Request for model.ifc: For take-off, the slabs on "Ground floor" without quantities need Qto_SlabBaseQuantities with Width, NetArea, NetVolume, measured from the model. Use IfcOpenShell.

First a look at what the model holds.

```python
import ifcopenshell
import ifcopenshell.util.element
import ifcopenshell.util.unit

model = ifcopenshell.open("model.ifc")
print(model.schema)
for unit_type in ("LENGTHUNIT", "AREAUNIT", "VOLUMEUNIT"):
    print(unit_type, ifcopenshell.util.unit.calculate_unit_scale(model, unit_type))
storey = next(s for s in model.by_type("IfcBuildingStorey") if s.Name == "Ground floor")
slabs = [e for e in ifcopenshell.util.element.get_decomposition(storey) if e.is_a("IfcSlab")]
for e in sorted(slabs, key=lambda e: e.id()):
    print(e.id(), e.is_a(), e.Name, list(ifcopenshell.util.element.get_psets(e, qtos_only=True)), sep=" | ")
```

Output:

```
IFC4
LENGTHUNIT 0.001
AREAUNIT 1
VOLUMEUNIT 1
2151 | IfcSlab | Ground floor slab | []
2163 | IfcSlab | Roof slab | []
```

```python
import ifcopenshell
import ifcopenshell.api.pset
import ifcopenshell.geom
import ifcopenshell.util.element
import ifcopenshell.util.shape
import ifcopenshell.util.unit

model = ifcopenshell.open("model.ifc")
unit_scale = ifcopenshell.util.unit.calculate_unit_scale(model)
area_scale = ifcopenshell.util.unit.calculate_unit_scale(model, "AREAUNIT")
volume_scale = ifcopenshell.util.unit.calculate_unit_scale(model, "VOLUMEUNIT")
settings = ifcopenshell.geom.settings()

storey = next(s for s in model.by_type("IfcBuildingStorey") if s.Name == "Ground floor")
slabs = [e for e in ifcopenshell.util.element.get_decomposition(storey) if e.is_a("IfcSlab")]

for e in sorted(slabs, key=lambda e: e.id()):
    if ifcopenshell.util.element.get_psets(e, qtos_only=True, should_inherit=False):
        continue
    # Geometry comes back in metres, in the element's own axes.
    shape = ifcopenshell.geom.create_shape(settings, e)
    values = {
        "Width": ifcopenshell.util.shape.get_z(shape.geometry) / unit_scale,
        "NetArea": ifcopenshell.util.shape.get_footprint_area(shape.geometry) / area_scale,
        "NetVolume": ifcopenshell.util.shape.get_volume(shape.geometry) / volume_scale,
    }
    qto = ifcopenshell.api.pset.add_qto(model, product=e, name="Qto_SlabBaseQuantities")
    ifcopenshell.api.pset.edit_qto(model, qto=qto, properties=values)
    print(e.id(), {k: round(v, 3) for k, v in values.items()})

model.write("model_rev.ifc")
```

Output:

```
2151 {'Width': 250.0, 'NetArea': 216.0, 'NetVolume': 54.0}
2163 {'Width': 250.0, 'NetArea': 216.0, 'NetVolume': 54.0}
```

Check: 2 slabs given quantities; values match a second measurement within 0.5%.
